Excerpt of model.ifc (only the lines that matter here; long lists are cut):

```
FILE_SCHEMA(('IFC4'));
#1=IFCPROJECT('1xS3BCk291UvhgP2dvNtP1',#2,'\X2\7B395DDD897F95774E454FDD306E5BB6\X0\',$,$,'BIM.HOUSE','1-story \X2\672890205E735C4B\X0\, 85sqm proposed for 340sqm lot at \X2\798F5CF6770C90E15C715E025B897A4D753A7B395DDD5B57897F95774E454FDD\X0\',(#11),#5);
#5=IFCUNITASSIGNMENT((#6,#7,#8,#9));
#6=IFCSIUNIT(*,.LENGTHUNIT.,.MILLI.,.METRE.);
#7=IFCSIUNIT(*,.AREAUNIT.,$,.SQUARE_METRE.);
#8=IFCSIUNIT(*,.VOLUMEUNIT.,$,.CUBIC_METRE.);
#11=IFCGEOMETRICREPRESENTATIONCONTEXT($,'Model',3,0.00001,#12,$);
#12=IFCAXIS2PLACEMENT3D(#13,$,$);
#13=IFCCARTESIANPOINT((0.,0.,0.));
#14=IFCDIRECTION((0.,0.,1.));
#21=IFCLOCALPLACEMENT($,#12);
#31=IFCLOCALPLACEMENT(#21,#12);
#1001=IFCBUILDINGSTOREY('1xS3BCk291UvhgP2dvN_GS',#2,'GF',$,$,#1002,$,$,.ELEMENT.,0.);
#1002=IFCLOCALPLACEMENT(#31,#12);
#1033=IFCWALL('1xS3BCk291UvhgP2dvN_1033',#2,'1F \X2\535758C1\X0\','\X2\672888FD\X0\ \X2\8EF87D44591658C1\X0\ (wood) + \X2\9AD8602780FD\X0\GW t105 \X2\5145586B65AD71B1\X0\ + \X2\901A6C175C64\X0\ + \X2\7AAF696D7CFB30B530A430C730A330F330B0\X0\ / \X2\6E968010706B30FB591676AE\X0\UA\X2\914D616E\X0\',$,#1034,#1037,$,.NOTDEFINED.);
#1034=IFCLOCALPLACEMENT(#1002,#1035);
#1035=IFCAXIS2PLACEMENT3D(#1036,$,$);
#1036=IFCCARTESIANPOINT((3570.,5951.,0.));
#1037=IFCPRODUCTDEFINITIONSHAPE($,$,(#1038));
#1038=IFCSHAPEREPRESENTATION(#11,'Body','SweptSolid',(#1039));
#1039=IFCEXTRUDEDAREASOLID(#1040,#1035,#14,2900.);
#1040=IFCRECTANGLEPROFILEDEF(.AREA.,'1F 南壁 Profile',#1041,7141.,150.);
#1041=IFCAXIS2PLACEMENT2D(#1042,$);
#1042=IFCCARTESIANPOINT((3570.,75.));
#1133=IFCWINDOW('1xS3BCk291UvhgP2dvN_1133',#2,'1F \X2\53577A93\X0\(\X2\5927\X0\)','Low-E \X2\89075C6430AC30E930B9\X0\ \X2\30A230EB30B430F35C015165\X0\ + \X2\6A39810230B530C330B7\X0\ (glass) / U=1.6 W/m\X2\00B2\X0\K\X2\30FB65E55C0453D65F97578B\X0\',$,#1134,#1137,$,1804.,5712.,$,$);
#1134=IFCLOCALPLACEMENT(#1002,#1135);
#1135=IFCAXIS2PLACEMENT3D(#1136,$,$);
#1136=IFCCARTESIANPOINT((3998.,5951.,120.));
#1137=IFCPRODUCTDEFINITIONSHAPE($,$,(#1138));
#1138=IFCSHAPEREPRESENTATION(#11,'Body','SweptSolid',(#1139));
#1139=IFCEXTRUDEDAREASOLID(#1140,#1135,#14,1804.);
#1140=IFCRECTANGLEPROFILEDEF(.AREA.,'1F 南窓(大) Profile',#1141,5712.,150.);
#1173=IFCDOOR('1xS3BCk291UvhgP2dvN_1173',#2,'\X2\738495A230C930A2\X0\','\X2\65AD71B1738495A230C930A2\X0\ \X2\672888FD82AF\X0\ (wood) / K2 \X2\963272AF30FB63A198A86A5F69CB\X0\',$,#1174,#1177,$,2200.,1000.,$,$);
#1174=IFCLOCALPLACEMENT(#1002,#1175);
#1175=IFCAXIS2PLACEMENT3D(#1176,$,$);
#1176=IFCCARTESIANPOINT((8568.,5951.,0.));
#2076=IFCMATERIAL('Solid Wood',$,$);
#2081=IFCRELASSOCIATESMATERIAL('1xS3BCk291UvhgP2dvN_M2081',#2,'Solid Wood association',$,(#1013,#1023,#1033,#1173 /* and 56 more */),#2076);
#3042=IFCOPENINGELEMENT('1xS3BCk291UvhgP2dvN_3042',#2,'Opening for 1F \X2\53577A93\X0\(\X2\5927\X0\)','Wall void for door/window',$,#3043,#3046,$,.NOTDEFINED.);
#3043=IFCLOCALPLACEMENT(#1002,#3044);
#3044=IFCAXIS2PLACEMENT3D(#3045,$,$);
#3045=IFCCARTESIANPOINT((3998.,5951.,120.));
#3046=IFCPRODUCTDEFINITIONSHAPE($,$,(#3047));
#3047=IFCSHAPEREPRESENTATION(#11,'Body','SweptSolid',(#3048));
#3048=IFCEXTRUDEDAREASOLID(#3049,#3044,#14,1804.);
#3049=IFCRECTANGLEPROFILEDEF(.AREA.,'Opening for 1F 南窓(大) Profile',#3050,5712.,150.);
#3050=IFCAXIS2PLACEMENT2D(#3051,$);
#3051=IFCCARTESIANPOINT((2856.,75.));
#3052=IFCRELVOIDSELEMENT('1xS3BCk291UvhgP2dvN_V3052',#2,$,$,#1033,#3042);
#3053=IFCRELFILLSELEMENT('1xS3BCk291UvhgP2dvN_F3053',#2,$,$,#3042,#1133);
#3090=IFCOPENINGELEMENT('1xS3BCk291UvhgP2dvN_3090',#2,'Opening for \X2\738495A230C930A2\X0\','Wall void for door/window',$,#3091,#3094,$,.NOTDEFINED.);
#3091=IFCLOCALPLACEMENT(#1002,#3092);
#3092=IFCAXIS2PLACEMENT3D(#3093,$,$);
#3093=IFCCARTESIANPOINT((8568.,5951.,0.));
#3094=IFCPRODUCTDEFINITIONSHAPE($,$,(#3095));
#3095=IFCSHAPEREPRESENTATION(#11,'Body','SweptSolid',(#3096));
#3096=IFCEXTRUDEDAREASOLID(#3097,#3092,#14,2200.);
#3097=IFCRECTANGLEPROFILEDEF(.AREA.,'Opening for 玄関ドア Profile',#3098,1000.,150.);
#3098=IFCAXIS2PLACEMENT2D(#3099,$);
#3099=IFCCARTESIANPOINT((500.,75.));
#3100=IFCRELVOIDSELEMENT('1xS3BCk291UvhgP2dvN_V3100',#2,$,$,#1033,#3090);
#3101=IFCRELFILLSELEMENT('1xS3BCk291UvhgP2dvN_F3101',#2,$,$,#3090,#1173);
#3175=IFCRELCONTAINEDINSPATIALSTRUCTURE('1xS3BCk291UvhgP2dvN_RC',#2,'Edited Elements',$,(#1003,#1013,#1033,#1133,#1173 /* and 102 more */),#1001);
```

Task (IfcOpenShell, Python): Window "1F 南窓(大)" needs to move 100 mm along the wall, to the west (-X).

```python
import ifcopenshell
import ifcopenshell.api.geometry
import ifcopenshell.util.placement
import ifcopenshell.util.unit

model = ifcopenshell.open("model.ifc")
unit_scale = ifcopenshell.util.unit.calculate_unit_scale(model)

window = model.by_guid("1xS3BCk291UvhgP2dvN_1133")
opening = window.FillsVoids[0].RelatingOpeningElement
wall = opening.VoidsElements[0].RelatingBuildingElement

wall_matrix = ifcopenshell.util.placement.get_local_placement(wall.ObjectPlacement)
shift = wall_matrix[:3, 0] * -0.1 / unit_scale
before = ifcopenshell.util.placement.get_local_placement(window.ObjectPlacement)[:3, 3].copy()

# The window is not placed relative to its opening, so move both.
for product in (opening, window):
    matrix = ifcopenshell.util.placement.get_local_placement(product.ObjectPlacement)
    matrix[:3, 3] += shift
    ifcopenshell.api.geometry.edit_object_placement(model, product=product, matrix=matrix, is_si=False)

after = ifcopenshell.util.placement.get_local_placement(window.ObjectPlacement)[:3, 3]
print("window moved by", (after - before).round(3) + 0.0)

model.write("model_rev.ifc")
```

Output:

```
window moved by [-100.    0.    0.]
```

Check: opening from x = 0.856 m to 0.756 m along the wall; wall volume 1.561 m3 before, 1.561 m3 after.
